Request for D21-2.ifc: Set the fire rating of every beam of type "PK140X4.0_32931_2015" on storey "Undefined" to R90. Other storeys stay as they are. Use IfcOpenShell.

First a look at what the model holds.

```python
import ifcopenshell
import ifcopenshell.util.element

model = ifcopenshell.open("D21-2.ifc")
print(model.schema)
storey = next(s for s in model.by_type("IfcBuildingStorey") if s.Name == "Undefined")
beams = [e for e in ifcopenshell.util.element.get_decomposition(storey) if e.is_a("IfcBeam")]
seen = {}
for e in beams:
    element_type = ifcopenshell.util.element.get_type(e)
    key = (element_type.Name if element_type != e and element_type else None, ifcopenshell.util.element.get_pset(e, "Pset_BeamCommon", "FireRating"))
    seen[key] = seen.get(key, 0) + 1
for (name, value), count in sorted(seen.items(), key=str):
    print(count, "x", name, "|", value)
```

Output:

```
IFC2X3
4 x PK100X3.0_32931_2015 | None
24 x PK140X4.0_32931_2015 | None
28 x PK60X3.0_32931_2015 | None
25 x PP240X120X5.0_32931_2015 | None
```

```python
import ifcopenshell
import ifcopenshell.api.pset
import ifcopenshell.util.element

model = ifcopenshell.open("D21-2.ifc")

storey = next(s for s in model.by_type("IfcBuildingStorey") if s.Name == "Undefined")
beams = [e for e in ifcopenshell.util.element.get_decomposition(storey) if e.is_a("IfcBeam")]

count = 0
for e in beams:
    element_type = ifcopenshell.util.element.get_type(e)
    if element_type in (None, e) or element_type.Name != "PK140X4.0_32931_2015":
        continue
    found = ifcopenshell.util.element.get_pset(e, "Pset_BeamCommon", should_inherit=False)
    if found:
        pset = model.by_id(found["id"])
        if len(ifcopenshell.util.element.get_elements_by_pset(pset)) > 1:
            pset = ifcopenshell.api.pset.unshare_pset(model, products=[e], pset=pset)[0]
    else:
        pset = ifcopenshell.api.pset.add_pset(model, product=e, name="Pset_BeamCommon")
    ifcopenshell.api.pset.edit_pset(model, pset=pset, properties={"FireRating": "R90"})
    count += 1

print(count, "beams updated")

model.write("D21-2_v2.ifc")
```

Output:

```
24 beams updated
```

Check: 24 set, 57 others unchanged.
